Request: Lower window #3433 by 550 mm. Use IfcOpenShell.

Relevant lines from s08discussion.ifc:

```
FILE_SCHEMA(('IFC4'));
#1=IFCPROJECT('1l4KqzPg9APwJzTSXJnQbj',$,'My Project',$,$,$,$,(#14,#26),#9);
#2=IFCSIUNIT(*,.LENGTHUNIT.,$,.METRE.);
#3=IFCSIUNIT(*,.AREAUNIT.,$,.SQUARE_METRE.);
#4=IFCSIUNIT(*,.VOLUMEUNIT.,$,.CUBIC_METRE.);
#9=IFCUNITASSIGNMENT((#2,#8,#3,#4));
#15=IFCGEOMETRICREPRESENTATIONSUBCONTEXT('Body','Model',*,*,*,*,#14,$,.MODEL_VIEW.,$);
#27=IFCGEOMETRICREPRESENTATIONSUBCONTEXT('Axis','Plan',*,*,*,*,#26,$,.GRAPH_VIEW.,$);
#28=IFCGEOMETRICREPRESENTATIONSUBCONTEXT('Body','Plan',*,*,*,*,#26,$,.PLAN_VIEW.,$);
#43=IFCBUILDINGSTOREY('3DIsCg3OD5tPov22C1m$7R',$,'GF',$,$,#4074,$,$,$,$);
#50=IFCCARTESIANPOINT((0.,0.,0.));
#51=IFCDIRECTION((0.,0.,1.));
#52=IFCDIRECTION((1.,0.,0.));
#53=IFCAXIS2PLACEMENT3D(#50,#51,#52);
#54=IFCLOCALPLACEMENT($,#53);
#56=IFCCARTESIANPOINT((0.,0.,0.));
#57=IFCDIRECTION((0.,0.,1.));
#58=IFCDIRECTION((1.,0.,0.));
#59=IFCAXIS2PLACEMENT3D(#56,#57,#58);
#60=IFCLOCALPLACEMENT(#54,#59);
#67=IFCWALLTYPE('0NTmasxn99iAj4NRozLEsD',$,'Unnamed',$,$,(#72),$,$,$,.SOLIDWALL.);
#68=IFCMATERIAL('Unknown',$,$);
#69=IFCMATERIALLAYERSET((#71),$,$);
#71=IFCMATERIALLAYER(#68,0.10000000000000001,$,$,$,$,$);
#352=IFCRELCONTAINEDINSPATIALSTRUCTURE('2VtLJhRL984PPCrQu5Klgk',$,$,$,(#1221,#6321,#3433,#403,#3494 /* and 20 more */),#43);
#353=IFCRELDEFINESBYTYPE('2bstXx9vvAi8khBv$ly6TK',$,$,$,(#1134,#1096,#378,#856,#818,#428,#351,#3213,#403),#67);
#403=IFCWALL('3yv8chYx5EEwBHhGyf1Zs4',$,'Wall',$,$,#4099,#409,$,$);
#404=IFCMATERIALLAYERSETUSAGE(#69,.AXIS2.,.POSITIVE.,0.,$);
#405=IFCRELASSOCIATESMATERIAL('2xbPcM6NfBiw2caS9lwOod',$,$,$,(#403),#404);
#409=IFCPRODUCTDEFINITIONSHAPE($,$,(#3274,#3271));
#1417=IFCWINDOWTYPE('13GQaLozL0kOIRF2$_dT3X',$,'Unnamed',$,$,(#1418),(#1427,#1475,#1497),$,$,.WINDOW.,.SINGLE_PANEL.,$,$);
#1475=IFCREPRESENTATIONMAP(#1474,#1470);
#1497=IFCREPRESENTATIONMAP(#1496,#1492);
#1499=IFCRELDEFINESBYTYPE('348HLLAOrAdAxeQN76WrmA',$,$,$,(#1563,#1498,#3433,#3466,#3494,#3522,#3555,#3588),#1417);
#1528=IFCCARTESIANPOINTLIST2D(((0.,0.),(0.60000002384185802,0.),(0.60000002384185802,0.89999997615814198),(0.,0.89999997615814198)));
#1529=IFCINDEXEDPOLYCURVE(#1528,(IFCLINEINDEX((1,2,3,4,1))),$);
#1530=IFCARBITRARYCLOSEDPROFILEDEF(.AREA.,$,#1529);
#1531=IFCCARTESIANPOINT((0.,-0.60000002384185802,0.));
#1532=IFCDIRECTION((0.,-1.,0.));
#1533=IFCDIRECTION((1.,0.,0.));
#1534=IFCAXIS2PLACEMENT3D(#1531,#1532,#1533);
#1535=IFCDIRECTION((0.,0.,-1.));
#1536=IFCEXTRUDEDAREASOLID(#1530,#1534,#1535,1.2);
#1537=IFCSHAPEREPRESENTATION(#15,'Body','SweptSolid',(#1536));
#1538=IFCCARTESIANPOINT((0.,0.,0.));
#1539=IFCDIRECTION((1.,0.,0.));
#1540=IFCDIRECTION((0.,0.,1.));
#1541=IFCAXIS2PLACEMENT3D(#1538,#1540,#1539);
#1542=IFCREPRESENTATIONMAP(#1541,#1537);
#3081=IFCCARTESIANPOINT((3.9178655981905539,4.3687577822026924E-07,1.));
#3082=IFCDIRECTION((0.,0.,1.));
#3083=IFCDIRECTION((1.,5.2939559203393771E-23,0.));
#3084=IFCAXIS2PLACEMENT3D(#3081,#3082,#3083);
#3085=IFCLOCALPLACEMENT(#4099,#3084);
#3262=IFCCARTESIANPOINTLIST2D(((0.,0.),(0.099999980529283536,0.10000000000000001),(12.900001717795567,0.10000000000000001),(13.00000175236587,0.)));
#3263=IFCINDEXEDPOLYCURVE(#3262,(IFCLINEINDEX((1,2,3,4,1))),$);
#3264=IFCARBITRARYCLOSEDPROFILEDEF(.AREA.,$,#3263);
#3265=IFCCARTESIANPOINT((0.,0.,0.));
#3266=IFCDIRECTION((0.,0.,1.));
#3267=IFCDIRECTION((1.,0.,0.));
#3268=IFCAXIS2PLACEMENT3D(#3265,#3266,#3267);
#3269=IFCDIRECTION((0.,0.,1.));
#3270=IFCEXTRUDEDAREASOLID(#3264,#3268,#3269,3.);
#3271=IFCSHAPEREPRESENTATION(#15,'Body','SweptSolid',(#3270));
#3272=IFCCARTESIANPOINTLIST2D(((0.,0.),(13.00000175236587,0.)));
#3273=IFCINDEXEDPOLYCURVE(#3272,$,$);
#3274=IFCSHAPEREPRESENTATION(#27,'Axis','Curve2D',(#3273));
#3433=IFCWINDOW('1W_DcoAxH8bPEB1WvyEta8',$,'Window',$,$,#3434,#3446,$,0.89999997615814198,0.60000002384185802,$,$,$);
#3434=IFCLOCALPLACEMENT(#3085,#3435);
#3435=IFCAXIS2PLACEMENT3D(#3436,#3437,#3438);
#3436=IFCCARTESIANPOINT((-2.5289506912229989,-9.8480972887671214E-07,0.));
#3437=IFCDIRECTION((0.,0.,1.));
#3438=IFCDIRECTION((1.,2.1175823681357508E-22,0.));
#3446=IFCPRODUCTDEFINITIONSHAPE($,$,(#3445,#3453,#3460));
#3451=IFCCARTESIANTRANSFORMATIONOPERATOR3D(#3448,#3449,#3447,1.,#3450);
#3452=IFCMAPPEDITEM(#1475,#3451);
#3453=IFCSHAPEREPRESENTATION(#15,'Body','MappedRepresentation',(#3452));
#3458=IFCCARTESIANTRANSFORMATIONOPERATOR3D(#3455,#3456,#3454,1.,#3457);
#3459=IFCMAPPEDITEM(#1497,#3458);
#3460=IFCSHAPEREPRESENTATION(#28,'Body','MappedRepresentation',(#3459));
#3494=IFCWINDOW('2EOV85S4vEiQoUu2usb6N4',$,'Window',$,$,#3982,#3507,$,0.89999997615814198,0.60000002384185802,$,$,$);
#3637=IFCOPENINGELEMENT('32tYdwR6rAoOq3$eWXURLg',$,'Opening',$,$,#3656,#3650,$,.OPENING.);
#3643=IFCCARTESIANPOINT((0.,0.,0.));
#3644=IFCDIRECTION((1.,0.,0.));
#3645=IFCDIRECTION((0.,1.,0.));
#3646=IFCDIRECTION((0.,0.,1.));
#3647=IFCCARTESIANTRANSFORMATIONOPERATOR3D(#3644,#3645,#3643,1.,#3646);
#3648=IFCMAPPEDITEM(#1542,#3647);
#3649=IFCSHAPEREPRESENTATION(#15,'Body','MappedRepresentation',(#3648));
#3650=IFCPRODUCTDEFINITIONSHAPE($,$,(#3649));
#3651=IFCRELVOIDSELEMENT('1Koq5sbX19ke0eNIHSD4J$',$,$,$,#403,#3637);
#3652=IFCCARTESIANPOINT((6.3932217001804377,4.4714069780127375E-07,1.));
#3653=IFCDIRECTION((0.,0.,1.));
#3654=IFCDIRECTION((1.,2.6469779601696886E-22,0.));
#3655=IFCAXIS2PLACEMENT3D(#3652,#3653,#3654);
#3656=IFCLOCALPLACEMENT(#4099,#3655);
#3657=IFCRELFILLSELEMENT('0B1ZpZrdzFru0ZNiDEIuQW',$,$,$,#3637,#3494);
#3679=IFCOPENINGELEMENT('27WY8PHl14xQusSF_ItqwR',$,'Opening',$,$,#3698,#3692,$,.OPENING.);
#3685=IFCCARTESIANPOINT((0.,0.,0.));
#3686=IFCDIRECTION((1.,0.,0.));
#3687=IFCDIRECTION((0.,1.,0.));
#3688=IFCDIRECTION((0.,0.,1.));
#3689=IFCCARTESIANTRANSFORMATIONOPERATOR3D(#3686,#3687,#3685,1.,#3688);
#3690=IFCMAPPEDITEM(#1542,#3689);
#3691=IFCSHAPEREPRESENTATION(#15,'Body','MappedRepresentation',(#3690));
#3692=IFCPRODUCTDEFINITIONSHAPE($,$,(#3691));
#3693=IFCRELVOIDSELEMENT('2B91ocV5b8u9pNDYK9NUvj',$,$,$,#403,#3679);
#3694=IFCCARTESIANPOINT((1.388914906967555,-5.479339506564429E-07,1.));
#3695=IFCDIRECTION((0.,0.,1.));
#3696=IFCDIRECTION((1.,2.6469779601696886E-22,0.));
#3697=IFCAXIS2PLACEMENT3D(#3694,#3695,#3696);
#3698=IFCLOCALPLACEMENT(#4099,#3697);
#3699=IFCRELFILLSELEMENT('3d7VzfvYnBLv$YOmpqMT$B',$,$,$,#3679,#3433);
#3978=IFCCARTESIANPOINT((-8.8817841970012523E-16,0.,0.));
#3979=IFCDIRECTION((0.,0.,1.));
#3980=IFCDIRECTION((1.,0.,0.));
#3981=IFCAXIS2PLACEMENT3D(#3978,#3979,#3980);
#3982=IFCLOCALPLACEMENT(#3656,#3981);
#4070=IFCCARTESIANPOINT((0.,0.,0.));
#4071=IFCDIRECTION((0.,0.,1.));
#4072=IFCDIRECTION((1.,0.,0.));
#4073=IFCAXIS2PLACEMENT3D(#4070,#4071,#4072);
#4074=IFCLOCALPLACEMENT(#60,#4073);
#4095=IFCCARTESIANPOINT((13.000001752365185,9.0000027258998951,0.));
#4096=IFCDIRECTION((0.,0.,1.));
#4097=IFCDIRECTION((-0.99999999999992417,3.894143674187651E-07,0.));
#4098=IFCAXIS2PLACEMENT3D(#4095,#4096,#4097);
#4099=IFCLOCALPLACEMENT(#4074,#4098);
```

```python
import numpy as np
import ifcopenshell
import ifcopenshell.api.geometry
import ifcopenshell.util.placement
import ifcopenshell.util.unit

model = ifcopenshell.open("s08discussion.ifc")
unit_scale = ifcopenshell.util.unit.calculate_unit_scale(model)

window = model.by_id(3433)
opening = window.FillsVoids[0].RelatingOpeningElement
dz = -0.55 / unit_scale

shift = np.array([0.0, 0.0, dz])
# The window is not placed relative to its opening, so move both.
for product in (opening, window):
    matrix = ifcopenshell.util.placement.get_local_placement(product.ObjectPlacement)
    matrix[:3, 3] += shift
    ifcopenshell.api.geometry.edit_object_placement(model, product=product, matrix=matrix, is_si=False)

print(f"moved by {dz * unit_scale:+.3f} m")

model.write("s08discussion_v2.ifc")
```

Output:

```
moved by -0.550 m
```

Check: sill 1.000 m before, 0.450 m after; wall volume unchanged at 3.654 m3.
